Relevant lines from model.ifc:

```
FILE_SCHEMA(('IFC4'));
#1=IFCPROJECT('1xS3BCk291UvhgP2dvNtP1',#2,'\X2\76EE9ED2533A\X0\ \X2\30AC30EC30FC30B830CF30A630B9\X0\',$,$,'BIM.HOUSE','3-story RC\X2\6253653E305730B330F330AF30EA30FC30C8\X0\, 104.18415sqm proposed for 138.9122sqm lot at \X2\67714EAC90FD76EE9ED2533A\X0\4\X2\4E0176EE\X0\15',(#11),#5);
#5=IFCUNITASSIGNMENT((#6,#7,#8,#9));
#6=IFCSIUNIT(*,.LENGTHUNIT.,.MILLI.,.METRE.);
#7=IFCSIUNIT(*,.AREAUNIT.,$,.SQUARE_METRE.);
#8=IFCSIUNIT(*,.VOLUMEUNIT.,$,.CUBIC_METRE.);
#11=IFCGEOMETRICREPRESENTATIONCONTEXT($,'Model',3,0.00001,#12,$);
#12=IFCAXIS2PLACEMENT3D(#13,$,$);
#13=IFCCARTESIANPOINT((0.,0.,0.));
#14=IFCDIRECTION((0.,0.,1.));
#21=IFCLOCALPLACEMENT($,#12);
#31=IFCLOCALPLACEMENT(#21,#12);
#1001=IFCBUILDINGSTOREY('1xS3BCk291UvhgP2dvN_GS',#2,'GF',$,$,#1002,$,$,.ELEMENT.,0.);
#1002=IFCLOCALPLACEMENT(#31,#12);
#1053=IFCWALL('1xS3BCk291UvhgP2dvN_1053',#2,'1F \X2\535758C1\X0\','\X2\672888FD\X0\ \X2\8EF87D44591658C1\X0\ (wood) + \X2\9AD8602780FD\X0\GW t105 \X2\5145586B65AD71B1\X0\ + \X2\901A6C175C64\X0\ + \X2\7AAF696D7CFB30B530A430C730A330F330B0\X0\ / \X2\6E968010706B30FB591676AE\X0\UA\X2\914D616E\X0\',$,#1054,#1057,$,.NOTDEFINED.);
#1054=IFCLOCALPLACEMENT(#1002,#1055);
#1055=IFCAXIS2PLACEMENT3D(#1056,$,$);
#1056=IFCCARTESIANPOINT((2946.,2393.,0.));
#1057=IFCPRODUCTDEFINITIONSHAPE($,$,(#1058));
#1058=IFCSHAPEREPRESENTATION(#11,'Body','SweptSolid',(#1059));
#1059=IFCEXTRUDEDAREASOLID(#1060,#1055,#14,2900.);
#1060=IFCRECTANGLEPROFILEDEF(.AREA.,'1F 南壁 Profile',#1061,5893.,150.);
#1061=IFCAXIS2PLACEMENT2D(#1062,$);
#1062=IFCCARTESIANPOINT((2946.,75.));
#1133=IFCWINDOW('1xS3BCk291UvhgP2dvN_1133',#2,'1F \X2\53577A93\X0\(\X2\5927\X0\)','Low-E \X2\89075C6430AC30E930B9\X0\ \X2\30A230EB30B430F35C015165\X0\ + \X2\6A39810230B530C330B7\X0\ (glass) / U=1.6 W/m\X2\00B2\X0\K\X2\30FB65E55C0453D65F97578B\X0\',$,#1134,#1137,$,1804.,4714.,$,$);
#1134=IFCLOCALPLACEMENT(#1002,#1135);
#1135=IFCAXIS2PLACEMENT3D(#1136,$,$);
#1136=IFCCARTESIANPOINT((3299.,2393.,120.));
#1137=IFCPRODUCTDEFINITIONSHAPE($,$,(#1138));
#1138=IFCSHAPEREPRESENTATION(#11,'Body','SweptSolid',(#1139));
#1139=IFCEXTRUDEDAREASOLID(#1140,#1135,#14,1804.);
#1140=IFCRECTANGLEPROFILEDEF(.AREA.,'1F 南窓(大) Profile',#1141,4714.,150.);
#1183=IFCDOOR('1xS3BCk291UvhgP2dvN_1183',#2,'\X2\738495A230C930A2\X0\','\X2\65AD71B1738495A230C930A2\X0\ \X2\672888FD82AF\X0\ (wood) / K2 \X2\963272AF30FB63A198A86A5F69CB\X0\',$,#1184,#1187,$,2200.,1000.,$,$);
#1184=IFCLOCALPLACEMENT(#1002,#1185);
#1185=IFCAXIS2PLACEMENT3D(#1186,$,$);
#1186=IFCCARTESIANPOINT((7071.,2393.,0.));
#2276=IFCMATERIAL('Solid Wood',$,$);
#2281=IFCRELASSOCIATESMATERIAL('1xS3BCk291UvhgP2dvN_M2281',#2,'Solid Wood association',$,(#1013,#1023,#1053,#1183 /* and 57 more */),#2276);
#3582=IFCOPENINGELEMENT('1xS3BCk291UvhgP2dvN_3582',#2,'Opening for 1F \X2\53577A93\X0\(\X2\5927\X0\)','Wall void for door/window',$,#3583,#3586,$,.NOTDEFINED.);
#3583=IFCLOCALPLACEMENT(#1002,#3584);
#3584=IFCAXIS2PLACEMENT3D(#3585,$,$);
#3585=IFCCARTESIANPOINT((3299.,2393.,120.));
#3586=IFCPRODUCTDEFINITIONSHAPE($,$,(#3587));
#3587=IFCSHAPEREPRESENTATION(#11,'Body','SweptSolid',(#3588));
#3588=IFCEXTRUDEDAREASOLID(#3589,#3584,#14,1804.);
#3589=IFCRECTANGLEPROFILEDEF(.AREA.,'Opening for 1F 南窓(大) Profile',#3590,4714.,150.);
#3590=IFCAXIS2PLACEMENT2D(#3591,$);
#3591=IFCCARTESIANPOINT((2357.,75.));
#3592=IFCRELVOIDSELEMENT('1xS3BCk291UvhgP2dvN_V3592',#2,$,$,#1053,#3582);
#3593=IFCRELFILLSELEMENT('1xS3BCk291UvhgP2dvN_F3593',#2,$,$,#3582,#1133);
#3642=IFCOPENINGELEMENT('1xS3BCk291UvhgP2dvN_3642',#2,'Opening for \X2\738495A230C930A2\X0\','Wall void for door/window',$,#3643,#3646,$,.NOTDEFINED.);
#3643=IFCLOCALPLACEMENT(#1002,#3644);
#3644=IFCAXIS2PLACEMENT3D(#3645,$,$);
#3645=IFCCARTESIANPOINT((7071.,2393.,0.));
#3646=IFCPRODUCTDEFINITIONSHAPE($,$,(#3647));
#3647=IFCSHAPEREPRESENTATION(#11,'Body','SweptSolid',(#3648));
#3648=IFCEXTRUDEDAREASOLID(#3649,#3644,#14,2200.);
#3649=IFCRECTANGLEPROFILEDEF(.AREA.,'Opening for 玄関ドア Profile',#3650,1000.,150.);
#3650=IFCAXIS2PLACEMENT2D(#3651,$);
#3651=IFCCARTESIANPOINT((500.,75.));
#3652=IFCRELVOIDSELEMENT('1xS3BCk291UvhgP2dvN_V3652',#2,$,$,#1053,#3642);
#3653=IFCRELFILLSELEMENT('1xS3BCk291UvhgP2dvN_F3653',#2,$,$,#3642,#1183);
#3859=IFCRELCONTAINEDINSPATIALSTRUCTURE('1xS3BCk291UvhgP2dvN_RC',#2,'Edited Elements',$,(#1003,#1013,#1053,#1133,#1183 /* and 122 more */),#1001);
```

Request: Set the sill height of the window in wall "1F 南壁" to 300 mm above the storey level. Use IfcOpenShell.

```python
import numpy as np
import ifcopenshell
import ifcopenshell.api.geometry
import ifcopenshell.geom
import ifcopenshell.util.element
import ifcopenshell.util.placement
import ifcopenshell.util.shape
import ifcopenshell.util.unit

model = ifcopenshell.open("model.ifc")
unit_scale = ifcopenshell.util.unit.calculate_unit_scale(model)

window = model.by_guid("1xS3BCk291UvhgP2dvN_1133")
opening = window.FillsVoids[0].RelatingOpeningElement
storey = ifcopenshell.util.element.get_container(window, ifc_class="IfcBuildingStorey")
level = ifcopenshell.util.placement.get_local_placement(storey.ObjectPlacement)[2, 3]

# The opening's origin need not be at the sill, so measure its lowest point.
shape = ifcopenshell.geom.create_shape(ifcopenshell.geom.settings(), opening)
bottom = ifcopenshell.util.shape.get_shape_bottom_elevation(shape, shape.geometry) / unit_scale
dz = level + 300.0 - bottom

shift = np.array([0.0, 0.0, dz])
# The window is not placed relative to its opening, so move both.
for product in (opening, window):
    matrix = ifcopenshell.util.placement.get_local_placement(product.ObjectPlacement)
    matrix[:3, 3] += shift
    ifcopenshell.api.geometry.edit_object_placement(model, product=product, matrix=matrix, is_si=False)

print(f"moved by {dz * unit_scale:+.3f} m")

model.write("model_updated.ifc")
```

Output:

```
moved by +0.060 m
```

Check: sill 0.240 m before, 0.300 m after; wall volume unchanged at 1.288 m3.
